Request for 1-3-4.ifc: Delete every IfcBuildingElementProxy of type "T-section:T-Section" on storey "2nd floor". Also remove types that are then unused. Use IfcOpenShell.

First a look at what the model holds.

```python
import ifcopenshell
import ifcopenshell.util.element

model = ifcopenshell.open("1-3-4.ifc")
print(model.schema)
storey = next(s for s in model.by_type("IfcBuildingStorey") if s.Name == "2nd floor")
proxies = [e for e in ifcopenshell.util.element.get_decomposition(storey) if e.is_a("IfcBuildingElementProxy")]
seen = {}
for e in proxies:
    element_type = ifcopenshell.util.element.get_type(e)
    name = element_type.Name if element_type not in (None, e) else None
    seen[name] = seen.get(name, 0) + 1
for name, count in sorted(seen.items(), key=str):
    print(count, "x", name)
```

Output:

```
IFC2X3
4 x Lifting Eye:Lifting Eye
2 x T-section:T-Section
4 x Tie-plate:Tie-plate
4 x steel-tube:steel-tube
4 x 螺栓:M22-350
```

```python
import ifcopenshell
import ifcopenshell.api.root
import ifcopenshell.util.element

model = ifcopenshell.open("1-3-4.ifc")

storey = next(s for s in model.by_type("IfcBuildingStorey") if s.Name == "2nd floor")
proxies = [e for e in ifcopenshell.util.element.get_decomposition(storey) if e.is_a("IfcBuildingElementProxy")]
targets = [e for e in proxies if (t := ifcopenshell.util.element.get_type(e)) not in (None, e) and t.Name == "T-section:T-Section"]
types = {ifcopenshell.util.element.get_type(e) for e in targets} - {None, *targets}

for e in targets:
    ifcopenshell.api.root.remove_product(model, product=e)
print(len(targets), "removed")

unused = [t for t in types if not ifcopenshell.util.element.get_types(t)]
for t in unused:
    ifcopenshell.api.root.remove_product(model, product=t)
print(len(unused), "unused types removed")

model.write("1-3-4_edited.ifc")
```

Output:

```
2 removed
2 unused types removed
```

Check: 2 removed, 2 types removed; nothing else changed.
